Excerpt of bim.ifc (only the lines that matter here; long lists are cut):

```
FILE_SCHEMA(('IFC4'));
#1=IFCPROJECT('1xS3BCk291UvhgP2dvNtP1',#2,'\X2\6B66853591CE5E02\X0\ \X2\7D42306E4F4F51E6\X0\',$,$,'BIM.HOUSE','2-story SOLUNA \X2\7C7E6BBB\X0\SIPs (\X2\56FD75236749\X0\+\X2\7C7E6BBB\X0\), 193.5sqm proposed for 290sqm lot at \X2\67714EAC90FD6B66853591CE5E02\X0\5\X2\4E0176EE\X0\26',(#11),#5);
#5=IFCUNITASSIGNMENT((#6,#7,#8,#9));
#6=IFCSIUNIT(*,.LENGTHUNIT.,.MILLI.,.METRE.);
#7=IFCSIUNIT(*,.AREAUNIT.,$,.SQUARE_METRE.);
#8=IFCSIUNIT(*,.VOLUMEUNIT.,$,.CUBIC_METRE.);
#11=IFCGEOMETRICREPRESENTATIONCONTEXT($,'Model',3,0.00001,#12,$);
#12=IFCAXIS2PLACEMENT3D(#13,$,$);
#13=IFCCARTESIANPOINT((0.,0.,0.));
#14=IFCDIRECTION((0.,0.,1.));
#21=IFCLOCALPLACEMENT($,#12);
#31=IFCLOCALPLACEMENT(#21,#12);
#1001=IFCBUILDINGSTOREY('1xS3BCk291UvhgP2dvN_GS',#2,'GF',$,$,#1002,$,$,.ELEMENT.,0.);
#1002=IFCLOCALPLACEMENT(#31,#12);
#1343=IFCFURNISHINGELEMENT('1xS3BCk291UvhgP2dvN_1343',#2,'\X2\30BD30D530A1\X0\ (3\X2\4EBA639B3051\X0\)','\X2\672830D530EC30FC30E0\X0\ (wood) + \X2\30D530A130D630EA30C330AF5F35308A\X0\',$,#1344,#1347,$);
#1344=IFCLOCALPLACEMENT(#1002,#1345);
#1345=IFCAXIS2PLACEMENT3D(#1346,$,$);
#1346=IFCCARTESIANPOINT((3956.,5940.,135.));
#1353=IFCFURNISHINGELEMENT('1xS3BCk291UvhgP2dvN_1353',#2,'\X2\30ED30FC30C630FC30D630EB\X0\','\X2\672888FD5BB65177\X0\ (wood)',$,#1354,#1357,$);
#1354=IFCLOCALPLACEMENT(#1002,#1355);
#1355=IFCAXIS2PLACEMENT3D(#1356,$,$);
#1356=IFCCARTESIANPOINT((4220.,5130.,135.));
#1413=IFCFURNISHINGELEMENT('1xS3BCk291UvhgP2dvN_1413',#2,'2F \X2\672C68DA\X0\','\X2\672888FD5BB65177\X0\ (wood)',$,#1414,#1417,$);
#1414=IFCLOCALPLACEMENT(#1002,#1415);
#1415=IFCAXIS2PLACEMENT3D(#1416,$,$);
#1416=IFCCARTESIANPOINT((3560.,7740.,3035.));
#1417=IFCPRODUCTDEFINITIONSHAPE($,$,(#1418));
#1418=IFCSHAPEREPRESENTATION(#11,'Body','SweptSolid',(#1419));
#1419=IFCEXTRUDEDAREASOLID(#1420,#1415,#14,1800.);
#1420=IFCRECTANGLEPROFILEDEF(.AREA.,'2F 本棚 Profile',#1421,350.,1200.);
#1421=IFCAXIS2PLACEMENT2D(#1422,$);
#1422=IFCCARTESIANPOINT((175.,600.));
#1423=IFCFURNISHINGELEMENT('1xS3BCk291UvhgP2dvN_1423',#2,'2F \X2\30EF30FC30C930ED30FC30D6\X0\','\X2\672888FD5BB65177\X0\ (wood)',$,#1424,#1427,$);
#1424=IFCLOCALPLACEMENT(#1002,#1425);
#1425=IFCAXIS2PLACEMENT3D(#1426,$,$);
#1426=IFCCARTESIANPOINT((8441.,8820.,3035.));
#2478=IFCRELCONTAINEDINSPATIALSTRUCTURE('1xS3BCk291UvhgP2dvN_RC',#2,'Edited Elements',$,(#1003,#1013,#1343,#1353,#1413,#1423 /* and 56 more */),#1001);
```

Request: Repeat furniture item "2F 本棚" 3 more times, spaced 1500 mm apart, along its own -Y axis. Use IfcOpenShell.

```python
import ifcopenshell
import ifcopenshell.api.geometry
import ifcopenshell.api.root
import ifcopenshell.util.element
import ifcopenshell.util.placement
import ifcopenshell.util.unit

model = ifcopenshell.open("bim.ifc")
unit_scale = ifcopenshell.util.unit.calculate_unit_scale(model)


def reuse_history(source, copy):
    """copy_class also copies each property set's owner history, people and application; keep the originals."""
    for rel in copy.IsDefinedBy:
        if rel.is_a("IfcRelDefinesByProperties") and (history := rel.RelatingPropertyDefinition.OwnerHistory):
            rel.RelatingPropertyDefinition.OwnerHistory = source.OwnerHistory
            ifcopenshell.util.element.remove_deep2(model, history)


source = model.by_id(1413)
base = ifcopenshell.util.placement.get_local_placement(source.ObjectPlacement)
step = -base[:3, 1] * 1.5 / unit_scale

for i in range(1, 4):
    copy = ifcopenshell.api.root.copy_class(model, product=source)
    copy.Representation = ifcopenshell.util.element.copy_deep(
        model, source.Representation, exclude=["IfcGeometricRepresentationContext", "IfcRepresentationMap"]
    )
    reuse_history(source, copy)
    matrix = base.copy()
    matrix[:3, 3] += i * step
    print("added at", matrix[:3, 3].round(3) + 0.0)
    ifcopenshell.api.geometry.edit_object_placement(model, product=copy, matrix=matrix, is_si=False)

model.write("bim-out.ifc")
```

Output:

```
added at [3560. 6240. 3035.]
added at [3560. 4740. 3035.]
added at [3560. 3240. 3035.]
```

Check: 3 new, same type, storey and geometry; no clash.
